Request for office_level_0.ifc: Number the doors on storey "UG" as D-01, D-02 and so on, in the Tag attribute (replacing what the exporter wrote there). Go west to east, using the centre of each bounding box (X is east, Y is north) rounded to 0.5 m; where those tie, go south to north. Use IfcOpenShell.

First a look at what the model holds.

```python
import ifcopenshell
import ifcopenshell.util.element
import ifcopenshell.util.placement

model = ifcopenshell.open("office_level_0.ifc")
print(model.schema)
storey = next(s for s in model.by_type("IfcBuildingStorey") if s.Name == "UG")
doors = [e for e in ifcopenshell.util.element.get_decomposition(storey) if e.is_a("IfcDoor")]
for e in sorted(doors, key=lambda e: e.id()):
    origin = ifcopenshell.util.placement.get_local_placement(e.ObjectPlacement)[:3, 3]
    print(e.id(), e.Tag, e.Name, origin.round(2) + 0.0, sep=" | ")
```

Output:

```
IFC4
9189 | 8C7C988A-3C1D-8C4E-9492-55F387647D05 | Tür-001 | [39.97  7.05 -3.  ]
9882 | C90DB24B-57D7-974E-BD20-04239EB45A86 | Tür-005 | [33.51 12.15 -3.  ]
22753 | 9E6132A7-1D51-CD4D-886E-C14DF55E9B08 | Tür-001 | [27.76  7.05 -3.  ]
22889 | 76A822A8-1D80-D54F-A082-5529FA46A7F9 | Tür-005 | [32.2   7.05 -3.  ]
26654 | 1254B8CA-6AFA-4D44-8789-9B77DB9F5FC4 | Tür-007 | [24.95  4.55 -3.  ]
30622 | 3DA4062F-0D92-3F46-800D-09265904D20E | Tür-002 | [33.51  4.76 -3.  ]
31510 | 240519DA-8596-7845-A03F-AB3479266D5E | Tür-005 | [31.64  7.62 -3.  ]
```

```python
import ifcopenshell
import ifcopenshell.geom
import ifcopenshell.util.element
import ifcopenshell.util.shape

model = ifcopenshell.open("office_level_0.ifc")
settings = ifcopenshell.geom.settings()
settings.set("use-world-coords", True)


def centre(element):
    shape = ifcopenshell.geom.create_shape(settings, element)
    return ifcopenshell.util.shape.get_bbox_centroid(shape.geometry)


storey = next(s for s in model.by_type("IfcBuildingStorey") if s.Name == "UG")
doors = [e for e in ifcopenshell.util.element.get_decomposition(storey) if e.is_a("IfcDoor")]

# Insertion points can sit at a corner or the storey origin, so sort by the geometry (in metres).
centres = {e: centre(e) for e in doors}
doors.sort(key=lambda e: (round(centres[e][0] / 0.5), centres[e][1]))

for i, e in enumerate(doors, start=1):
    number = f"D-{i:02d}"
    e.Tag = number
    print(e.id(), number)

model.write("office_level_0_rev.ifc")
```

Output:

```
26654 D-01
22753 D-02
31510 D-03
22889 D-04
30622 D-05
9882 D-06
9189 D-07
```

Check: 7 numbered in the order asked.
